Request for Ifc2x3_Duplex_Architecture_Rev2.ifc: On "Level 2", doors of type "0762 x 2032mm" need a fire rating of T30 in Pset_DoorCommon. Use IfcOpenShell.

First a look at what the model holds.

```python
import ifcopenshell
import ifcopenshell.util.element

model = ifcopenshell.open("Ifc2x3_Duplex_Architecture_Rev2.ifc")
print(model.schema)
storey = next(s for s in model.by_type("IfcBuildingStorey") if s.Name == "Level 2")
doors = [e for e in ifcopenshell.util.element.get_decomposition(storey) if e.is_a("IfcDoor")]
seen = {}
for e in doors:
    element_type = ifcopenshell.util.element.get_type(e)
    key = (element_type.Name if element_type != e and element_type else None, ifcopenshell.util.element.get_pset(e, "Pset_DoorCommon", "FireRating"))
    seen[key] = seen.get(key, 0) + 1
for (name, value), count in sorted(seen.items(), key=str):
    print(count, "x", name, "|", value)
```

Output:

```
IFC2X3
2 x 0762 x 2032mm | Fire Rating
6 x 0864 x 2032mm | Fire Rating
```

```python
import ifcopenshell
import ifcopenshell.api.pset
import ifcopenshell.util.element

model = ifcopenshell.open("Ifc2x3_Duplex_Architecture_Rev2.ifc")

storey = next(s for s in model.by_type("IfcBuildingStorey") if s.Name == "Level 2")
doors = [e for e in ifcopenshell.util.element.get_decomposition(storey) if e.is_a("IfcDoor")]

count = 0
for e in doors:
    element_type = ifcopenshell.util.element.get_type(e)
    if element_type in (None, e) or element_type.Name != "0762 x 2032mm":
        continue
    # add_pset returns the element's existing set when there is one.
    pset = ifcopenshell.api.pset.add_pset(model, product=e, name="Pset_DoorCommon")
    ifcopenshell.api.pset.edit_pset(model, pset=pset, properties={"FireRating": "T30"})
    count += 1

print(count, "doors updated")

model.write("Ifc2x3_Duplex_Architecture_Rev2_edited.ifc")
```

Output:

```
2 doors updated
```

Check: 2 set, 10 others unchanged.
